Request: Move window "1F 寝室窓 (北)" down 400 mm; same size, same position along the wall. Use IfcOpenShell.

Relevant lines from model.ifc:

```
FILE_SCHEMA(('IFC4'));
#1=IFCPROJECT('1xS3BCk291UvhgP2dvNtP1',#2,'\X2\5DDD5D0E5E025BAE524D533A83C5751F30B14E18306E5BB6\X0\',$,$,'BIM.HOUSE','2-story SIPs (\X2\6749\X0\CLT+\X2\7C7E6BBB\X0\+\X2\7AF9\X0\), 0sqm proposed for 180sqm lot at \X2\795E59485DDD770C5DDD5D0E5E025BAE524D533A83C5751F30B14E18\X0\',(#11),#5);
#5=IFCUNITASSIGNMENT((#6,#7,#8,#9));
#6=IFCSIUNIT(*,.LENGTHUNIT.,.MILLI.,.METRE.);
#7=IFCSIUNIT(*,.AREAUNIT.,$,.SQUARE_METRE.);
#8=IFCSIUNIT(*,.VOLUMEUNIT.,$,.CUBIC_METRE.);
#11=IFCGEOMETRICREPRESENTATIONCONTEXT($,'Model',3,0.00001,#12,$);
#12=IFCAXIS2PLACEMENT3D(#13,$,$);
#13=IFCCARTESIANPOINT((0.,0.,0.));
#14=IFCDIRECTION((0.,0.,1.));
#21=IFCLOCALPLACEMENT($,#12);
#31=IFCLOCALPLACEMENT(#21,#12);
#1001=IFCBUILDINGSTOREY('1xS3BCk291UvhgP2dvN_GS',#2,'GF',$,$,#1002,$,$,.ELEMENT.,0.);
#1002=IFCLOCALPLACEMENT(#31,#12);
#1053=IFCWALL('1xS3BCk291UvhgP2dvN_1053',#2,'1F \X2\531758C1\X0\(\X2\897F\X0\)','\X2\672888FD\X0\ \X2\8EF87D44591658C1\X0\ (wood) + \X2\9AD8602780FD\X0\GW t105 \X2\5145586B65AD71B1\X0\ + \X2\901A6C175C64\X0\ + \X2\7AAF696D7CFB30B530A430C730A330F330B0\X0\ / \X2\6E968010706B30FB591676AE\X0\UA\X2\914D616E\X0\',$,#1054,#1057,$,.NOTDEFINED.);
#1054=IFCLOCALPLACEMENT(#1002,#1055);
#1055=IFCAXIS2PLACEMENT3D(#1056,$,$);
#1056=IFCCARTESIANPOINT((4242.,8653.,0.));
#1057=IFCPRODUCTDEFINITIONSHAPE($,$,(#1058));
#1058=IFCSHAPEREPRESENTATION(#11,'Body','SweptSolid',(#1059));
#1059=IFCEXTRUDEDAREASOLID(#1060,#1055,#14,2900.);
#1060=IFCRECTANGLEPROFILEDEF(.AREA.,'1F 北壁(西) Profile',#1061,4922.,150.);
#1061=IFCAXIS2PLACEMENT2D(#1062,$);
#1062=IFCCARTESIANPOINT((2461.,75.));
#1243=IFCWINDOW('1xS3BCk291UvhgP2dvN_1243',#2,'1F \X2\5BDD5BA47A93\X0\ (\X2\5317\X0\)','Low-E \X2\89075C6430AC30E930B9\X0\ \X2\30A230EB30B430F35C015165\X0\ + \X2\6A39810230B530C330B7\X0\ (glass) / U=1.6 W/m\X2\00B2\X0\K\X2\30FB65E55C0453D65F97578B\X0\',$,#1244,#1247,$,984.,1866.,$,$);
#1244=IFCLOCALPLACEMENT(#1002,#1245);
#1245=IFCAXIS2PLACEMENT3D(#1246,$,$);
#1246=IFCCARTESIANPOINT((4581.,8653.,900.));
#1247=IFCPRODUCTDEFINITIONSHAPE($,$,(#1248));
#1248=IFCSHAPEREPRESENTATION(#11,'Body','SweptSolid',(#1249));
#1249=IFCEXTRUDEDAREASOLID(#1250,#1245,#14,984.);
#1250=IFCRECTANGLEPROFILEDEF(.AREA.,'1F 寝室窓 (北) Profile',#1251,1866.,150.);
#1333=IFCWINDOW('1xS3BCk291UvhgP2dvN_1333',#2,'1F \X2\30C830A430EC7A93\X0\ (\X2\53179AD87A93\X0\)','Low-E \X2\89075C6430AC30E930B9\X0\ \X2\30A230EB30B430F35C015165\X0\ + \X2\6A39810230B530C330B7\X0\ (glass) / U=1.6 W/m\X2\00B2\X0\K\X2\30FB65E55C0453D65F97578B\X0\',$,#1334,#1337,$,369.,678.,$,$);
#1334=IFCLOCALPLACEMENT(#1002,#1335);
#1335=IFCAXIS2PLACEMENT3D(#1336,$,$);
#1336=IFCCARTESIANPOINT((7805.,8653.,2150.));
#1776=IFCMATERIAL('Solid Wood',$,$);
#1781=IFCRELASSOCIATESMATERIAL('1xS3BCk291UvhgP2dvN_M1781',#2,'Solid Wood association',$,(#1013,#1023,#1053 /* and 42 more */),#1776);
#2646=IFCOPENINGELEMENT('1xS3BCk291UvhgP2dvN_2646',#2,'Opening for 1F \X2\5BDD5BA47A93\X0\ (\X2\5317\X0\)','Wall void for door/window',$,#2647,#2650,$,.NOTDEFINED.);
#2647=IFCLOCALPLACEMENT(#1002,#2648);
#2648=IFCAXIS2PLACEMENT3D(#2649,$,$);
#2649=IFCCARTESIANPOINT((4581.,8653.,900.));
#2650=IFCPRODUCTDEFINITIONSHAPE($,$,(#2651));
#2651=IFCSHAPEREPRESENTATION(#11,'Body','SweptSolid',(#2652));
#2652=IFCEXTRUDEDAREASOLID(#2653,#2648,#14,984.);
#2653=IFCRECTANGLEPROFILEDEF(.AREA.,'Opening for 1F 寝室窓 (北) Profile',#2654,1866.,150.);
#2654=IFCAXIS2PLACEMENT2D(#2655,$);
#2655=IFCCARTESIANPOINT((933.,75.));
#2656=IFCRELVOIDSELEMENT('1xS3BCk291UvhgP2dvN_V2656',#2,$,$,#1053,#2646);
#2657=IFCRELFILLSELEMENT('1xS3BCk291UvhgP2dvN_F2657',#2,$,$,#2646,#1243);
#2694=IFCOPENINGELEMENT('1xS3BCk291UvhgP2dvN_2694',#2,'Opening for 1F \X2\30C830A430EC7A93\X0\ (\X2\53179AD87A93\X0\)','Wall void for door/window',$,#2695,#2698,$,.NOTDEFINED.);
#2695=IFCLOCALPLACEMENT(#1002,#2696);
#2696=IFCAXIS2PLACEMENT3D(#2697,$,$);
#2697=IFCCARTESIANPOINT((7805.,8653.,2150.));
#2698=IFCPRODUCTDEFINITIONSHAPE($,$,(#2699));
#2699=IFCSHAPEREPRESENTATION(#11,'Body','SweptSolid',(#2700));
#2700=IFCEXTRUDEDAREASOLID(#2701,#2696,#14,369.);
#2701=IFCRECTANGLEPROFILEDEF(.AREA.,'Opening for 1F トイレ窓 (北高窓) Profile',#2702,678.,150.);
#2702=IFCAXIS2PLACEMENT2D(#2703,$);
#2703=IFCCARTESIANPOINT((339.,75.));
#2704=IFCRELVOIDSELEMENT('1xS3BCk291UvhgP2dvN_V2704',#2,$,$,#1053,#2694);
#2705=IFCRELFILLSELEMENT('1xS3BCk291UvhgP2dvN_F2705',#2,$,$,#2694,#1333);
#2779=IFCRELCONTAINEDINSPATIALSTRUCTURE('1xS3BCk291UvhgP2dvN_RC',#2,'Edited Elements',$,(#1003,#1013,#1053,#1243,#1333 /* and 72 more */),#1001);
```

```python
import numpy as np
import ifcopenshell
import ifcopenshell.api.geometry
import ifcopenshell.util.placement
import ifcopenshell.util.unit

model = ifcopenshell.open("model.ifc")
unit_scale = ifcopenshell.util.unit.calculate_unit_scale(model)

window = model.by_id(1243)
opening = window.FillsVoids[0].RelatingOpeningElement
dz = -400.0

shift = np.array([0.0, 0.0, dz])
# The window is not placed relative to its opening, so move both.
for product in (opening, window):
    matrix = ifcopenshell.util.placement.get_local_placement(product.ObjectPlacement)
    matrix[:3, 3] += shift
    ifcopenshell.api.geometry.edit_object_placement(model, product=product, matrix=matrix, is_si=False)

print(f"moved by {dz * unit_scale:+.3f} m")

model.write("model_rev.ifc")
```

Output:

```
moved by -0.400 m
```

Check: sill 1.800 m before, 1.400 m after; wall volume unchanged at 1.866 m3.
